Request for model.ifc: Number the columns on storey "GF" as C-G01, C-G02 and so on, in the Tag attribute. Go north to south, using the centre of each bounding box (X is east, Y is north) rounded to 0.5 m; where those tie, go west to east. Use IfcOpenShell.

First a look at what the model holds.

```python
import ifcopenshell
import ifcopenshell.util.element
import ifcopenshell.util.placement

model = ifcopenshell.open("model.ifc")
print(model.schema)
storey = next(s for s in model.by_type("IfcBuildingStorey") if s.Name == "GF")
columns = [e for e in ifcopenshell.util.element.get_decomposition(storey) if e.is_a("IfcColumn")]
for e in sorted(columns, key=lambda e: e.id()):
    origin = ifcopenshell.util.placement.get_local_placement(e.ObjectPlacement)[:3, 3]
    print(e.id(), e.Tag, e.Name, origin.round(2) + 0.0, sep=" | ")
```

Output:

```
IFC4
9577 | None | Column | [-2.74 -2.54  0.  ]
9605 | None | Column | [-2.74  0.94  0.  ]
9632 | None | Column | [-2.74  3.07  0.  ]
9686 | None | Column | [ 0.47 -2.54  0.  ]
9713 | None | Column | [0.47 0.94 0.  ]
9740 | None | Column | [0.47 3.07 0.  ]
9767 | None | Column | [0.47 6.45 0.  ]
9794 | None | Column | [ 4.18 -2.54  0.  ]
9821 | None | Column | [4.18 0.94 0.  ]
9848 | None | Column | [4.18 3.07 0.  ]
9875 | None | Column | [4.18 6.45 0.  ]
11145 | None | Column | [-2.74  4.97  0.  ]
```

```python
import ifcopenshell
import ifcopenshell.geom
import ifcopenshell.util.element
import ifcopenshell.util.shape

model = ifcopenshell.open("model.ifc")
settings = ifcopenshell.geom.settings()
settings.set("use-world-coords", True)


def centre(element):
    shape = ifcopenshell.geom.create_shape(settings, element)
    return ifcopenshell.util.shape.get_bbox_centroid(shape.geometry)


storey = next(s for s in model.by_type("IfcBuildingStorey") if s.Name == "GF")
columns = [e for e in ifcopenshell.util.element.get_decomposition(storey) if e.is_a("IfcColumn")]

# Insertion points can sit at a corner or the storey origin, so sort by the geometry (in metres).
centres = {e: centre(e) for e in columns}
columns.sort(key=lambda e: (-round(centres[e][1] / 0.5), centres[e][0]))

for i, e in enumerate(columns, start=1):
    number = f"C-G{i:02d}"
    e.Tag = number
    print(e.id(), number)

model.write("model_edited.ifc")
```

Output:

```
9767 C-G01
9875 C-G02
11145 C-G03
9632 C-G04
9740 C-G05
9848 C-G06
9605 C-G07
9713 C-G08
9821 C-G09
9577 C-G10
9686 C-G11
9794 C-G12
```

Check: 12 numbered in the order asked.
